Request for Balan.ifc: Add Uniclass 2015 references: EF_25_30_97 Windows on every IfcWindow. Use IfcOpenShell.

First a look at what the model holds.

```python
import ifcopenshell

model = ifcopenshell.open("Balan.ifc")
print(model.schema)
print("classifications:", [c.Name for c in model.by_type("IfcClassification")])
for ifc_class in ("IfcDoor", "IfcRoof", "IfcStair", "IfcWall", "IfcWindow"):
    print(ifc_class, len(model.by_type(ifc_class)))
```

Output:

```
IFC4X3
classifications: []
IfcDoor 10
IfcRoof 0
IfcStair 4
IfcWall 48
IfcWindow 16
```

```python
import ifcopenshell
import ifcopenshell.api.classification

model = ifcopenshell.open("Balan.ifc")

system = ifcopenshell.api.classification.add_classification(model, classification="Uniclass 2015")

codes = {
    "IfcWindow": ("EF_25_30_97", "Windows"),
}
for ifc_class, (code, name) in codes.items():
    products = model.by_type(ifc_class)
    ifcopenshell.api.classification.add_reference(
        model, products=products, classification=system, identification=code, name=name
    )
    print(code, len(products))

model.write("Balan-out.ifc")
```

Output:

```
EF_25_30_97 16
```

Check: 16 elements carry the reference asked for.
